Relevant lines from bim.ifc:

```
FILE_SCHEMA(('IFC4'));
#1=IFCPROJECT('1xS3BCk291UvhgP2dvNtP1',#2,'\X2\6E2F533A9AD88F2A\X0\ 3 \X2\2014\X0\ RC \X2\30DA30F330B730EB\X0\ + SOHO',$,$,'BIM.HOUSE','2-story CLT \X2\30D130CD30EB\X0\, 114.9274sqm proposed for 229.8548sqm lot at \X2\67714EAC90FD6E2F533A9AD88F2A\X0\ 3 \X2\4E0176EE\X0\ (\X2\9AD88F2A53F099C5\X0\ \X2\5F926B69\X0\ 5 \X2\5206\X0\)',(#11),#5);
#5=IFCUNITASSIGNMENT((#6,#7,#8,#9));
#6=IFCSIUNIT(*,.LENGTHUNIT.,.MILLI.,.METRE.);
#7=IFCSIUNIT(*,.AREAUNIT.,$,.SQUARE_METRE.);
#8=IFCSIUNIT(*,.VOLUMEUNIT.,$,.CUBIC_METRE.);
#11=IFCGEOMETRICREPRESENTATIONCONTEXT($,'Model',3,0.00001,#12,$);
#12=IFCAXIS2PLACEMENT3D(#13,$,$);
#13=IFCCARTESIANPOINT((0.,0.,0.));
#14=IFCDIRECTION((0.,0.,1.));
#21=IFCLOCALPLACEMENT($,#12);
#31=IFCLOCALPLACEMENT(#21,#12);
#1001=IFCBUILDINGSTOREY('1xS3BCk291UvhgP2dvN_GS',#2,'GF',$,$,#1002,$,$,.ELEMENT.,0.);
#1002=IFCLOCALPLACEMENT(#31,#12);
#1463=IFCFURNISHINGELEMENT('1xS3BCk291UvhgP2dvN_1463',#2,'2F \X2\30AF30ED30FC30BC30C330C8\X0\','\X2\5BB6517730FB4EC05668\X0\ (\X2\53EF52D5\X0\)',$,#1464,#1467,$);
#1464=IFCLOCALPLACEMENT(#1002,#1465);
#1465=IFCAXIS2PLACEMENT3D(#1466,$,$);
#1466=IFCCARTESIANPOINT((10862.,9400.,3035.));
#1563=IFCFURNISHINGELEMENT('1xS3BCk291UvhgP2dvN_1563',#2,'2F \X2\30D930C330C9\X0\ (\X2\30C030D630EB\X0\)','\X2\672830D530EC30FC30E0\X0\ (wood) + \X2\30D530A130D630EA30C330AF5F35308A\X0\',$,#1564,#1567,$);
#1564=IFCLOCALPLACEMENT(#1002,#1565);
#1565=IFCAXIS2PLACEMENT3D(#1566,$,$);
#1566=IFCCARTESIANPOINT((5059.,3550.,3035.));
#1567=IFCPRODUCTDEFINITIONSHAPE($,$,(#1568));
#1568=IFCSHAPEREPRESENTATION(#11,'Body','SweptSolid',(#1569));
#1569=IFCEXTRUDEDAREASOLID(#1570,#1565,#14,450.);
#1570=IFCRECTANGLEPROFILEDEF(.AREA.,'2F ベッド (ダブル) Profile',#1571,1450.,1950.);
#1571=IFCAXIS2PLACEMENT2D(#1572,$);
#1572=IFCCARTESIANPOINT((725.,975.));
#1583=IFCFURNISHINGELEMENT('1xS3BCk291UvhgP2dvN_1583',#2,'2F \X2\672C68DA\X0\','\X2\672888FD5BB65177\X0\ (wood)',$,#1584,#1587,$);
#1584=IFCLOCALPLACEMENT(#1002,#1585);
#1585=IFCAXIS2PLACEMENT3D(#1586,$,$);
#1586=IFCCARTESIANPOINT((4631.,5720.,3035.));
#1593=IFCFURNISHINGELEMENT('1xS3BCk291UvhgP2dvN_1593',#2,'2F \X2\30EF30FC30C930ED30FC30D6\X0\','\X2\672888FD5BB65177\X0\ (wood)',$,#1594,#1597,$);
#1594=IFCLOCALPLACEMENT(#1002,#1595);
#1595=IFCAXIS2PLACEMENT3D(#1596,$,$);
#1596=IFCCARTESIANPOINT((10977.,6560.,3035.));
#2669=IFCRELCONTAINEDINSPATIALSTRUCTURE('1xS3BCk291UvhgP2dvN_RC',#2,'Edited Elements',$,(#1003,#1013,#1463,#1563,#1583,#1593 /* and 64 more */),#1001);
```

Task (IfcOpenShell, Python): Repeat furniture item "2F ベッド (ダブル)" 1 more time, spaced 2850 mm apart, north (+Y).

```python
import numpy as np
import ifcopenshell
import ifcopenshell.api.geometry
import ifcopenshell.api.root
import ifcopenshell.util.element
import ifcopenshell.util.placement
import ifcopenshell.util.unit

model = ifcopenshell.open("bim.ifc")
unit_scale = ifcopenshell.util.unit.calculate_unit_scale(model)


def reuse_history(source, copy):
    """copy_class also copies each property set's owner history, people and application; keep the originals."""
    for rel in copy.IsDefinedBy:
        if rel.is_a("IfcRelDefinesByProperties") and (history := rel.RelatingPropertyDefinition.OwnerHistory):
            rel.RelatingPropertyDefinition.OwnerHistory = source.OwnerHistory
            ifcopenshell.util.element.remove_deep2(model, history)


source = model.by_guid("1xS3BCk291UvhgP2dvN_1563")
base = ifcopenshell.util.placement.get_local_placement(source.ObjectPlacement)
step = np.array([0.0, 1.0, 0.0]) * 2.85 / unit_scale

for i in range(1, 2):
    copy = ifcopenshell.api.root.copy_class(model, product=source)
    copy.Representation = ifcopenshell.util.element.copy_deep(
        model, source.Representation, exclude=["IfcGeometricRepresentationContext", "IfcRepresentationMap"]
    )
    reuse_history(source, copy)
    matrix = base.copy()
    matrix[:3, 3] += i * step
    print("added at", matrix[:3, 3].round(3) + 0.0)
    ifcopenshell.api.geometry.edit_object_placement(model, product=copy, matrix=matrix, is_si=False)

model.write("bim_v2.ifc")
```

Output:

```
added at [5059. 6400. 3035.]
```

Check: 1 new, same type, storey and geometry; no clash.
